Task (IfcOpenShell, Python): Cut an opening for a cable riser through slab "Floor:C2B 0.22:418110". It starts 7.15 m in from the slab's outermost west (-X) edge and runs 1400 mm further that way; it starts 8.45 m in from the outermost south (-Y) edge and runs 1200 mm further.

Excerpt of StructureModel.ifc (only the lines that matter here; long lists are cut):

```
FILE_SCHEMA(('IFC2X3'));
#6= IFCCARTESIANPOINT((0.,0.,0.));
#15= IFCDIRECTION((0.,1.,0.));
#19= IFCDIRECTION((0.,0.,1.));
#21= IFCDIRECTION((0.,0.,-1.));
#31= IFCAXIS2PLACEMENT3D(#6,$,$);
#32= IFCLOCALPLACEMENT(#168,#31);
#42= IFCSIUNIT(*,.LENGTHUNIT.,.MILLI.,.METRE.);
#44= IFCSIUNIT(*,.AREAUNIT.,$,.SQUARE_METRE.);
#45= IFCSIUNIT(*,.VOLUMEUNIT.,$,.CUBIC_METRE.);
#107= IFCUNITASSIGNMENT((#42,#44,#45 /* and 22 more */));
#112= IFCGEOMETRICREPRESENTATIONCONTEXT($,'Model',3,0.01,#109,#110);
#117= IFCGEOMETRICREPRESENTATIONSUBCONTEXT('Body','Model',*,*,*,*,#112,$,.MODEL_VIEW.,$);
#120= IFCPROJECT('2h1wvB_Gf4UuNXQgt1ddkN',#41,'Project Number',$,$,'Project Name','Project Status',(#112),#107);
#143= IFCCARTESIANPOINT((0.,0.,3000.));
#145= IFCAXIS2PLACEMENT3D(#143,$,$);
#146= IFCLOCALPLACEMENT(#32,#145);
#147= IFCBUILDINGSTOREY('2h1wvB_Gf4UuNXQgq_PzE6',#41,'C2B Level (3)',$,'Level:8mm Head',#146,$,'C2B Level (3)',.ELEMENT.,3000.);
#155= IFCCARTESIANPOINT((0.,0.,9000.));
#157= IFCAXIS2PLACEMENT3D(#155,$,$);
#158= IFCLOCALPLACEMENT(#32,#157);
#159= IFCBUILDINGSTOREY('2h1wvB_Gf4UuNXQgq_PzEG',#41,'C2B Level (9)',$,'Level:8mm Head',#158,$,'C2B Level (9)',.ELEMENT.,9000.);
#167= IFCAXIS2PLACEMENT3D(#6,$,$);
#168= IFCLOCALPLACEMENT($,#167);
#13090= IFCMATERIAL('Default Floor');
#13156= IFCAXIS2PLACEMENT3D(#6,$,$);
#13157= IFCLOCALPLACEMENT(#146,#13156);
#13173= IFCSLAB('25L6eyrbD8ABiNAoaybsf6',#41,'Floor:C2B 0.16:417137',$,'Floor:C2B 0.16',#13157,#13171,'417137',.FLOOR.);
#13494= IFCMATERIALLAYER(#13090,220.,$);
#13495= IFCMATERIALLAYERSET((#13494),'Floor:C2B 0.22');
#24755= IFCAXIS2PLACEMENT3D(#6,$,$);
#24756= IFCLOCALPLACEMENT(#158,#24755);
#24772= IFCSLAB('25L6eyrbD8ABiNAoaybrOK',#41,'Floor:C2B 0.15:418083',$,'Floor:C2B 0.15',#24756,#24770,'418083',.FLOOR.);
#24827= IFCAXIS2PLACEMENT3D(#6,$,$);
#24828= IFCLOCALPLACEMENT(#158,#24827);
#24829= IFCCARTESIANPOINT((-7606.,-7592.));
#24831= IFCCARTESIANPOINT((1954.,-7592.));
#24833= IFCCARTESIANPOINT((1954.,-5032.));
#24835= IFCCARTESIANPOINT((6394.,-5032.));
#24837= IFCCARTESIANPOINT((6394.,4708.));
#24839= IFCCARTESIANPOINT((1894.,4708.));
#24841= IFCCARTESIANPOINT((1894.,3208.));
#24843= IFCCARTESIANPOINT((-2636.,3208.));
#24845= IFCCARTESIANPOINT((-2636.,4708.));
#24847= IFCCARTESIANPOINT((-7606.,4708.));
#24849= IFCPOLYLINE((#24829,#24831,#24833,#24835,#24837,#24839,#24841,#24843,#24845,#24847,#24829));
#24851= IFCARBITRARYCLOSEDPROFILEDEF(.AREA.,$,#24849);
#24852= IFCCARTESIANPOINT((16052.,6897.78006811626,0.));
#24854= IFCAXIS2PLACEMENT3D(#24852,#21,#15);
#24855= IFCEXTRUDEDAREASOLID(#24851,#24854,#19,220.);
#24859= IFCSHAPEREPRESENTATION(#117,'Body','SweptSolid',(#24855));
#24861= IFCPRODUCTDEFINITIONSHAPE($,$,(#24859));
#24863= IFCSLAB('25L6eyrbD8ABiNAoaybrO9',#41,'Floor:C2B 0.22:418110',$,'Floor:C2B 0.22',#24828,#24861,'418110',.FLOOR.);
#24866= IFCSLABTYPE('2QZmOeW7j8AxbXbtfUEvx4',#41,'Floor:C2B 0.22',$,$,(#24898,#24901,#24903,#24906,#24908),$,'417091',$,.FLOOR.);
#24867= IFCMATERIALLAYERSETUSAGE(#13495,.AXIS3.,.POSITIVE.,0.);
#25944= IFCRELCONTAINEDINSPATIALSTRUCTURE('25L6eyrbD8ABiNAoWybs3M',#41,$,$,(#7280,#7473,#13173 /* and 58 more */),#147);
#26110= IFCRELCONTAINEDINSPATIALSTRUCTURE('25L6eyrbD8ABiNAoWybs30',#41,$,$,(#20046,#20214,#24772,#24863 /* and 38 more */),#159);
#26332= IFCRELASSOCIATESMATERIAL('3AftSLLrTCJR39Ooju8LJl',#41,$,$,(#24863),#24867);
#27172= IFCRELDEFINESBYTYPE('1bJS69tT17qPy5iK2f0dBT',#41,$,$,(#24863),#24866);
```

```python
import numpy as np
import ifcopenshell
import ifcopenshell.api.feature
import ifcopenshell.api.geometry
import ifcopenshell.api.root
import ifcopenshell.geom
import ifcopenshell.util.placement
import ifcopenshell.util.representation
import ifcopenshell.util.shape
import ifcopenshell.util.unit

model = ifcopenshell.open("StructureModel.ifc")
unit_scale = ifcopenshell.util.unit.calculate_unit_scale(model)
settings = ifcopenshell.geom.settings()


def volume(element):
    """Net volume in cubic metres, openings subtracted."""
    shape = ifcopenshell.geom.create_shape(settings, element)
    return ifcopenshell.util.shape.get_volume(shape.geometry)


slab = model.by_guid("25L6eyrbD8ABiNAoaybrO9")
before = volume(slab)

# Extent in the slab's own axes, in metres. The edges named are its -X and -Y sides.
slab_shape = ifcopenshell.geom.create_shape(settings, slab)
vertices = ifcopenshell.util.shape.get_vertices(slab_shape.geometry)
x_min, y_min, bottom = vertices.min(axis=0)
top = vertices[:, 2].max()

opening = ifcopenshell.api.root.create_entity(model, ifc_class="IfcOpeningElement", name="Cable riser opening")
context = ifcopenshell.util.representation.get_context(model, "Model", "Body", "MODEL_VIEW")
width, depth = 1.4, 1.2
outline = [(0.0, 0.0), (width, 0.0), (width, depth), (0.0, depth), (0.0, 0.0)]
# Overshoot both faces by 50 mm so the cut is clean.
shape = ifcopenshell.api.geometry.add_slab_representation(
    model, context=context, depth=top - bottom + 0.1, polyline=outline
)
ifcopenshell.api.geometry.assign_representation(model, product=opening, representation=shape)

matrix = ifcopenshell.util.placement.get_local_placement(slab.ObjectPlacement)
matrix[:, 3] = matrix @ np.append(np.array([x_min + 7.15, y_min + 8.45, bottom - 0.05]) / unit_scale, 1.0)
ifcopenshell.api.geometry.edit_object_placement(model, product=opening, matrix=matrix, is_si=False)
ifcopenshell.api.feature.add_feature(model, feature=opening, element=slab)

after = volume(slab)

print(f"slab volume {before:.3f} -> {after:.3f} m3")

model.write("StructureModel_edited.ifc")
```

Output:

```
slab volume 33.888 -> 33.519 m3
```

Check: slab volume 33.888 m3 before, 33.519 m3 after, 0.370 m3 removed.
